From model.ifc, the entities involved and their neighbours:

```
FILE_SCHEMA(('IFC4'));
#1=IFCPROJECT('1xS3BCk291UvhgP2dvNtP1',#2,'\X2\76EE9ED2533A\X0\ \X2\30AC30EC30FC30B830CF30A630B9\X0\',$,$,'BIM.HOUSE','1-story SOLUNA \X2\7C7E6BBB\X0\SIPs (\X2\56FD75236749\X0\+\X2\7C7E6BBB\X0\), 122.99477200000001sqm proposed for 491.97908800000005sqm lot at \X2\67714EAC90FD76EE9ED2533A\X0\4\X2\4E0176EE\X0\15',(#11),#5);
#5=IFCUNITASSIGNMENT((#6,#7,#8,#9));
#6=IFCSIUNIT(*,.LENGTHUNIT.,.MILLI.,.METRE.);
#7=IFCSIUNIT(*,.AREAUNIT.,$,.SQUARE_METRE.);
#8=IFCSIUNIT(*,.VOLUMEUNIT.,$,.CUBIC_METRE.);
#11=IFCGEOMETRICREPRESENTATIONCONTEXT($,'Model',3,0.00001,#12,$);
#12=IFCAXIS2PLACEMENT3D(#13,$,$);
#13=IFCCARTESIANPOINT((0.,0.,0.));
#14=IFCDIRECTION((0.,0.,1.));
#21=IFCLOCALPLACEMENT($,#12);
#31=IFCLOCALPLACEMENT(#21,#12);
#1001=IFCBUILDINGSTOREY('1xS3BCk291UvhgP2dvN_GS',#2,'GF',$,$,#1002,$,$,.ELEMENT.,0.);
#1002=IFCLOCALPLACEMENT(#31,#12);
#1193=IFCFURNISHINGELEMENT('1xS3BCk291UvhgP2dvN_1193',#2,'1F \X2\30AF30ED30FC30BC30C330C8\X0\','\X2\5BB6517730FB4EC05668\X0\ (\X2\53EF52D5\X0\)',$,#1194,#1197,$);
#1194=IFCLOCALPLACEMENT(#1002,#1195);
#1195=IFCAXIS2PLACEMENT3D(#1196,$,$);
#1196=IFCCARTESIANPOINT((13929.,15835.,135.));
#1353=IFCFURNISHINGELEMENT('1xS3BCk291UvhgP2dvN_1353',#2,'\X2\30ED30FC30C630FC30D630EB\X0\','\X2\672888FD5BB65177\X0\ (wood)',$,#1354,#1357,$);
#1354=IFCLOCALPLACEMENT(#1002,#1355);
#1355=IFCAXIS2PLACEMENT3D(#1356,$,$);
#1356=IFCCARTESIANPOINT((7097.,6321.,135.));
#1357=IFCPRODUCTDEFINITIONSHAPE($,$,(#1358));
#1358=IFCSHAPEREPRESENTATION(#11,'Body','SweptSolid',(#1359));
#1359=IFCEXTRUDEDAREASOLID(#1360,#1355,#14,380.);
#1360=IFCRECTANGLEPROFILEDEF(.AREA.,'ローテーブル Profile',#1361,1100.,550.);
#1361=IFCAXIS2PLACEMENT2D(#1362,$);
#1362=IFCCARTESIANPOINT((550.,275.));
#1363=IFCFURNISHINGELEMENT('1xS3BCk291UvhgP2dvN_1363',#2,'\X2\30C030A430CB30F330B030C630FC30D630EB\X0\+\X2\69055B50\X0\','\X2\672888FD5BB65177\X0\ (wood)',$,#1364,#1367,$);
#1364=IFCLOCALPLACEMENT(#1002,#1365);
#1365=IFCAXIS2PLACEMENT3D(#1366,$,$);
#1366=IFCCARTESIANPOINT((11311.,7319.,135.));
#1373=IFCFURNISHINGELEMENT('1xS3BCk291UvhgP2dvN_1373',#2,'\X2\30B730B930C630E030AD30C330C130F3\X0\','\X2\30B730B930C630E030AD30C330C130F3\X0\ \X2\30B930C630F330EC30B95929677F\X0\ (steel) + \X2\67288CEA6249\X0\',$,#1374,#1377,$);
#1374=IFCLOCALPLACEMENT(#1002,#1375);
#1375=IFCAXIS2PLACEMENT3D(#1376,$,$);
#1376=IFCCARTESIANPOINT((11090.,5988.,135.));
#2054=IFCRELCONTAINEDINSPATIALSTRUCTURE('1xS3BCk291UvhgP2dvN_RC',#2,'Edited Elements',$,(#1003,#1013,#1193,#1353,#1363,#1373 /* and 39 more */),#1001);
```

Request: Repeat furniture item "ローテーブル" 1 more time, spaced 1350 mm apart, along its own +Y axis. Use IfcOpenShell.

```python
import ifcopenshell
import ifcopenshell.api.geometry
import ifcopenshell.api.root
import ifcopenshell.util.element
import ifcopenshell.util.placement
import ifcopenshell.util.unit

model = ifcopenshell.open("model.ifc")
unit_scale = ifcopenshell.util.unit.calculate_unit_scale(model)


def reuse_history(source, copy):
    """copy_class also copies each property set's owner history, people and application; keep the originals."""
    for rel in copy.IsDefinedBy:
        if rel.is_a("IfcRelDefinesByProperties") and (history := rel.RelatingPropertyDefinition.OwnerHistory):
            rel.RelatingPropertyDefinition.OwnerHistory = source.OwnerHistory
            ifcopenshell.util.element.remove_deep2(model, history)


source = model.by_guid("1xS3BCk291UvhgP2dvN_1353")
base = ifcopenshell.util.placement.get_local_placement(source.ObjectPlacement)
step = base[:3, 1] * 1.35 / unit_scale

for i in range(1, 2):
    copy = ifcopenshell.api.root.copy_class(model, product=source)
    copy.Representation = ifcopenshell.util.element.copy_deep(
        model, source.Representation, exclude=["IfcGeometricRepresentationContext", "IfcRepresentationMap"]
    )
    reuse_history(source, copy)
    matrix = base.copy()
    matrix[:3, 3] += i * step
    print("added at", matrix[:3, 3].round(3) + 0.0)
    ifcopenshell.api.geometry.edit_object_placement(model, product=copy, matrix=matrix, is_si=False)

model.write("model_edited.ifc")
```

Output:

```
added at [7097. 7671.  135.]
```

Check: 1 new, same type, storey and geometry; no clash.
